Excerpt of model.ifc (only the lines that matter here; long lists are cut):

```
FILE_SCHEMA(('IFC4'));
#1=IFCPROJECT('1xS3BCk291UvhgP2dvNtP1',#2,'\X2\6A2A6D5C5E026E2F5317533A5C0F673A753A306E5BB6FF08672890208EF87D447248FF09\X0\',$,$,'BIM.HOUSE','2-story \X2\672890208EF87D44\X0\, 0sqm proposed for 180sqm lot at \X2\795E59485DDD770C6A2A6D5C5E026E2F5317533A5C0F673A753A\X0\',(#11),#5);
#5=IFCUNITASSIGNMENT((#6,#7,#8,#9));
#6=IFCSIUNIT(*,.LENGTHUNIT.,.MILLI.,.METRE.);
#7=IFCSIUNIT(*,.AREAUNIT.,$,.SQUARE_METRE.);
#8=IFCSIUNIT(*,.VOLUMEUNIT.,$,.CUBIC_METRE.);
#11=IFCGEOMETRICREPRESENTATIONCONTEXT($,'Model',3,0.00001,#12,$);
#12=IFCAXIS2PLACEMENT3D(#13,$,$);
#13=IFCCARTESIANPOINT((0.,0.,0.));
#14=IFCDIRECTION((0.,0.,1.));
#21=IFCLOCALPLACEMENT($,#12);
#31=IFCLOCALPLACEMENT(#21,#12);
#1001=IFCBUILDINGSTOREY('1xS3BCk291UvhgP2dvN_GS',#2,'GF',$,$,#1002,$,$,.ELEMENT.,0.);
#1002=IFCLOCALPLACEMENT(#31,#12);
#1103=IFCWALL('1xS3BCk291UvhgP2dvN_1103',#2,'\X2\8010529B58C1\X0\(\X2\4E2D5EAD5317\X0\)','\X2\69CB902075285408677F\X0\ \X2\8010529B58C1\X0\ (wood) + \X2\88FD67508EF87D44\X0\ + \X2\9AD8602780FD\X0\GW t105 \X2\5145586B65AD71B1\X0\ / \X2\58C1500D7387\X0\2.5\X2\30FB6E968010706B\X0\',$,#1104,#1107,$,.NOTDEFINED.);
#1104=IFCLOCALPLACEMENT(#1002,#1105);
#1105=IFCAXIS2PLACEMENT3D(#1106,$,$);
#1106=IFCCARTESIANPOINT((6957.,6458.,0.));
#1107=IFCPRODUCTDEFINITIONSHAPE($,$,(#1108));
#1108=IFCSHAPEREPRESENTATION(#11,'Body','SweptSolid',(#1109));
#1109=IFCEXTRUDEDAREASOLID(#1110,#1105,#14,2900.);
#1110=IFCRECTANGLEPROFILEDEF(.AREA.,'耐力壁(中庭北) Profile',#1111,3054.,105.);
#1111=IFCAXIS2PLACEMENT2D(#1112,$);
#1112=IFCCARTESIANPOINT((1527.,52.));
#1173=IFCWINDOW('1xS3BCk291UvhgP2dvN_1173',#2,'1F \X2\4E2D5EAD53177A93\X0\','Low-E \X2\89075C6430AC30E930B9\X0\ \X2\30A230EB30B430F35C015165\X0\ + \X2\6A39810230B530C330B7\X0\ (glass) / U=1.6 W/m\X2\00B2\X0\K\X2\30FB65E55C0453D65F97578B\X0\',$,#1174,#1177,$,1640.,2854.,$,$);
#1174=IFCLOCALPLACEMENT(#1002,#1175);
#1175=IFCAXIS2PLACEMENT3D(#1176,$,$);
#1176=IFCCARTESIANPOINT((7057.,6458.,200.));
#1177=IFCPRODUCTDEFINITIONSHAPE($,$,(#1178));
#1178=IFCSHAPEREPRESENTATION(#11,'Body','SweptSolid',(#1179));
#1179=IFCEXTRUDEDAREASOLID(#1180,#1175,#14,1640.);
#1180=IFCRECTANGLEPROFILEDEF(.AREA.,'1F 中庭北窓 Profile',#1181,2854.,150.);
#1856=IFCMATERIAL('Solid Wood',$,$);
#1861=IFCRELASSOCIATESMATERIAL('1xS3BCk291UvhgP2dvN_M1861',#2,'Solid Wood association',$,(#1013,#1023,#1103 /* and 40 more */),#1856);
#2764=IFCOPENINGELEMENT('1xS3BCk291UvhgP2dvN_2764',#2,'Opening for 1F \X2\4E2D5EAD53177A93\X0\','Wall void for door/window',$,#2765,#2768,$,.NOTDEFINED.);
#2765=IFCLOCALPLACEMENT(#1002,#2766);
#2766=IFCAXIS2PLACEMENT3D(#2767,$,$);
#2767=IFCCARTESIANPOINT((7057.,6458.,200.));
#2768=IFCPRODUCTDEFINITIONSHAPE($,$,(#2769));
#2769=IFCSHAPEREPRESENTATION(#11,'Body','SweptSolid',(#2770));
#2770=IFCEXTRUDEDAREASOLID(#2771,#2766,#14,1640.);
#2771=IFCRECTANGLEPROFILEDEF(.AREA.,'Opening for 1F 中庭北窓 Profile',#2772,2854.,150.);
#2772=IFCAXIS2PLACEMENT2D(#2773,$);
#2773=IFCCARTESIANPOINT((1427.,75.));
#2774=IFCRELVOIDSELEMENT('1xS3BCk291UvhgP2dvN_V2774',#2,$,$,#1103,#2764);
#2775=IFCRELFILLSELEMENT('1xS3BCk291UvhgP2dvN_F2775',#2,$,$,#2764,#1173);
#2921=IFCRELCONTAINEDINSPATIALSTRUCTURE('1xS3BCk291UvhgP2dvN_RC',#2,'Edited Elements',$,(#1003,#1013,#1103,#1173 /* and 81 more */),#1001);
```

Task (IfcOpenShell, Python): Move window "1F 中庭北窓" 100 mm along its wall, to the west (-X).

```python
import ifcopenshell
import ifcopenshell.api.geometry
import ifcopenshell.util.placement

model = ifcopenshell.open("model.ifc")

window = model.by_guid("1xS3BCk291UvhgP2dvN_1173")
opening = window.FillsVoids[0].RelatingOpeningElement
wall = opening.VoidsElements[0].RelatingBuildingElement

wall_matrix = ifcopenshell.util.placement.get_local_placement(wall.ObjectPlacement)
shift = wall_matrix[:3, 0] * -100.0
before = ifcopenshell.util.placement.get_local_placement(window.ObjectPlacement)[:3, 3].copy()

# The window is not placed relative to its opening, so move both.
for product in (opening, window):
    matrix = ifcopenshell.util.placement.get_local_placement(product.ObjectPlacement)
    matrix[:3, 3] += shift
    ifcopenshell.api.geometry.edit_object_placement(model, product=product, matrix=matrix, is_si=False)

after = ifcopenshell.util.placement.get_local_placement(window.ObjectPlacement)[:3, 3]
print("window moved by", (after - before).round(3) + 0.0)

model.write("model_updated.ifc")
```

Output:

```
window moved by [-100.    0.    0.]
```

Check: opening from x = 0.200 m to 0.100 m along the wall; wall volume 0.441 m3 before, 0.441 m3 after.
